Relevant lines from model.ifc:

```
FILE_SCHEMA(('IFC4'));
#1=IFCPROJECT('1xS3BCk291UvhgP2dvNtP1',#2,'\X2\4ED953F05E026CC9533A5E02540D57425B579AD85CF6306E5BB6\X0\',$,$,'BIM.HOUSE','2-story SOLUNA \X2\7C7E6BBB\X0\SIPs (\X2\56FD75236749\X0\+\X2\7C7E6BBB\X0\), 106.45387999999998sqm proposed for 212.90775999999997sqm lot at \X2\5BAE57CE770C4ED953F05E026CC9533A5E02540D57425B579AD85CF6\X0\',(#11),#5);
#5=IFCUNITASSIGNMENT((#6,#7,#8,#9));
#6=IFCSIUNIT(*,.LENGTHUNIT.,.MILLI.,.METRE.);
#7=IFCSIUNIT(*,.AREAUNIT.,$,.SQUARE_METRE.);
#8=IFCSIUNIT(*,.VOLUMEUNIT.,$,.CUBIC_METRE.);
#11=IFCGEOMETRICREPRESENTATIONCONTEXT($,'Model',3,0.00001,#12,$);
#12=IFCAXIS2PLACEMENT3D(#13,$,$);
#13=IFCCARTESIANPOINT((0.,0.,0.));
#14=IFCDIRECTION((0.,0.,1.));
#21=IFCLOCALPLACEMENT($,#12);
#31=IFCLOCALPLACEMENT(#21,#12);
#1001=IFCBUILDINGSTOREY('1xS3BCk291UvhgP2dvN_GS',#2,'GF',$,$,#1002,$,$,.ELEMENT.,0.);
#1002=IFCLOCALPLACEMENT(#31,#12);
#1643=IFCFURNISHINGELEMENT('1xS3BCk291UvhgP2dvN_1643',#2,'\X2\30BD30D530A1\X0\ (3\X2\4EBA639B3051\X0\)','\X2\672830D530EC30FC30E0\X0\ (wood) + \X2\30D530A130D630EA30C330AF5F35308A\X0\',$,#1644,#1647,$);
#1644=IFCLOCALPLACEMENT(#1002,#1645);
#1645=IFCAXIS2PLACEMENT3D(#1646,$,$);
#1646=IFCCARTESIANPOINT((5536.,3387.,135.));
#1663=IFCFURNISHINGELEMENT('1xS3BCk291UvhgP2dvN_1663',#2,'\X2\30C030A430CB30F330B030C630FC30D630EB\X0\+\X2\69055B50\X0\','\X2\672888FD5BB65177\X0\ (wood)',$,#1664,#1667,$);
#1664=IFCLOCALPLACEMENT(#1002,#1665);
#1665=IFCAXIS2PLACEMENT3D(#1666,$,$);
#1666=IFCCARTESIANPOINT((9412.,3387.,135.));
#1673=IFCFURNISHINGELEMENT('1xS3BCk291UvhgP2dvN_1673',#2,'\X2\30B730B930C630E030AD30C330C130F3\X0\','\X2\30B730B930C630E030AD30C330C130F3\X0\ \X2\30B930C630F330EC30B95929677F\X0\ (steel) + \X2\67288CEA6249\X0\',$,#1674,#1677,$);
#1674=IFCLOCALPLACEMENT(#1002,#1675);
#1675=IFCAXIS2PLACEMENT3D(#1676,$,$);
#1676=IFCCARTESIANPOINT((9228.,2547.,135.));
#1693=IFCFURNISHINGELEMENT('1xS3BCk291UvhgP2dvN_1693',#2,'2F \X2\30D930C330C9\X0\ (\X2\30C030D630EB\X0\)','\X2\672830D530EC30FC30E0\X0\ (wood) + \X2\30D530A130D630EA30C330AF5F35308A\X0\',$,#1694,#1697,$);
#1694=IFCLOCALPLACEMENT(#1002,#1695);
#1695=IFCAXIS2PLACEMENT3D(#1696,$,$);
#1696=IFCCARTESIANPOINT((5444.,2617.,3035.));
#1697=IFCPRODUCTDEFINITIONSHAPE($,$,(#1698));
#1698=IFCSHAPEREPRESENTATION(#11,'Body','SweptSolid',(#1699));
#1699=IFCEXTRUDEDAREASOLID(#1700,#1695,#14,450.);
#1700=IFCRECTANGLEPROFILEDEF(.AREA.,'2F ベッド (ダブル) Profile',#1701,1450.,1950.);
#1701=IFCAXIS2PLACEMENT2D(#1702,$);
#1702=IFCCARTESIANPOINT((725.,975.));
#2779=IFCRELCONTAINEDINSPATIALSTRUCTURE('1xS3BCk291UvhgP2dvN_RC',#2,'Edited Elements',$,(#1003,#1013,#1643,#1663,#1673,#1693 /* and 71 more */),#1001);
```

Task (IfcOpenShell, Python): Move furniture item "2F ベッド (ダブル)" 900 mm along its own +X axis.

```python
import ifcopenshell
import ifcopenshell.api.geometry
import ifcopenshell.util.placement

model = ifcopenshell.open("model.ifc")

item = model.by_id(1693)
matrix = ifcopenshell.util.placement.get_local_placement(item.ObjectPlacement)
matrix[:3, 3] += matrix[:3, 0] * 900.0
ifcopenshell.api.geometry.edit_object_placement(model, product=item, matrix=matrix, is_si=False)

print(ifcopenshell.util.placement.get_local_placement(item.ObjectPlacement).round(3) + 0.0)

model.write("model-out.ifc")
```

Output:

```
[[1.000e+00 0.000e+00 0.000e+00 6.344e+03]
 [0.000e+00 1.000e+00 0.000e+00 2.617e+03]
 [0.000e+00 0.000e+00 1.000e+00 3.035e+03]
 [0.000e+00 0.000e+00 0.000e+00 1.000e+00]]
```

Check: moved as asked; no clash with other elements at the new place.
